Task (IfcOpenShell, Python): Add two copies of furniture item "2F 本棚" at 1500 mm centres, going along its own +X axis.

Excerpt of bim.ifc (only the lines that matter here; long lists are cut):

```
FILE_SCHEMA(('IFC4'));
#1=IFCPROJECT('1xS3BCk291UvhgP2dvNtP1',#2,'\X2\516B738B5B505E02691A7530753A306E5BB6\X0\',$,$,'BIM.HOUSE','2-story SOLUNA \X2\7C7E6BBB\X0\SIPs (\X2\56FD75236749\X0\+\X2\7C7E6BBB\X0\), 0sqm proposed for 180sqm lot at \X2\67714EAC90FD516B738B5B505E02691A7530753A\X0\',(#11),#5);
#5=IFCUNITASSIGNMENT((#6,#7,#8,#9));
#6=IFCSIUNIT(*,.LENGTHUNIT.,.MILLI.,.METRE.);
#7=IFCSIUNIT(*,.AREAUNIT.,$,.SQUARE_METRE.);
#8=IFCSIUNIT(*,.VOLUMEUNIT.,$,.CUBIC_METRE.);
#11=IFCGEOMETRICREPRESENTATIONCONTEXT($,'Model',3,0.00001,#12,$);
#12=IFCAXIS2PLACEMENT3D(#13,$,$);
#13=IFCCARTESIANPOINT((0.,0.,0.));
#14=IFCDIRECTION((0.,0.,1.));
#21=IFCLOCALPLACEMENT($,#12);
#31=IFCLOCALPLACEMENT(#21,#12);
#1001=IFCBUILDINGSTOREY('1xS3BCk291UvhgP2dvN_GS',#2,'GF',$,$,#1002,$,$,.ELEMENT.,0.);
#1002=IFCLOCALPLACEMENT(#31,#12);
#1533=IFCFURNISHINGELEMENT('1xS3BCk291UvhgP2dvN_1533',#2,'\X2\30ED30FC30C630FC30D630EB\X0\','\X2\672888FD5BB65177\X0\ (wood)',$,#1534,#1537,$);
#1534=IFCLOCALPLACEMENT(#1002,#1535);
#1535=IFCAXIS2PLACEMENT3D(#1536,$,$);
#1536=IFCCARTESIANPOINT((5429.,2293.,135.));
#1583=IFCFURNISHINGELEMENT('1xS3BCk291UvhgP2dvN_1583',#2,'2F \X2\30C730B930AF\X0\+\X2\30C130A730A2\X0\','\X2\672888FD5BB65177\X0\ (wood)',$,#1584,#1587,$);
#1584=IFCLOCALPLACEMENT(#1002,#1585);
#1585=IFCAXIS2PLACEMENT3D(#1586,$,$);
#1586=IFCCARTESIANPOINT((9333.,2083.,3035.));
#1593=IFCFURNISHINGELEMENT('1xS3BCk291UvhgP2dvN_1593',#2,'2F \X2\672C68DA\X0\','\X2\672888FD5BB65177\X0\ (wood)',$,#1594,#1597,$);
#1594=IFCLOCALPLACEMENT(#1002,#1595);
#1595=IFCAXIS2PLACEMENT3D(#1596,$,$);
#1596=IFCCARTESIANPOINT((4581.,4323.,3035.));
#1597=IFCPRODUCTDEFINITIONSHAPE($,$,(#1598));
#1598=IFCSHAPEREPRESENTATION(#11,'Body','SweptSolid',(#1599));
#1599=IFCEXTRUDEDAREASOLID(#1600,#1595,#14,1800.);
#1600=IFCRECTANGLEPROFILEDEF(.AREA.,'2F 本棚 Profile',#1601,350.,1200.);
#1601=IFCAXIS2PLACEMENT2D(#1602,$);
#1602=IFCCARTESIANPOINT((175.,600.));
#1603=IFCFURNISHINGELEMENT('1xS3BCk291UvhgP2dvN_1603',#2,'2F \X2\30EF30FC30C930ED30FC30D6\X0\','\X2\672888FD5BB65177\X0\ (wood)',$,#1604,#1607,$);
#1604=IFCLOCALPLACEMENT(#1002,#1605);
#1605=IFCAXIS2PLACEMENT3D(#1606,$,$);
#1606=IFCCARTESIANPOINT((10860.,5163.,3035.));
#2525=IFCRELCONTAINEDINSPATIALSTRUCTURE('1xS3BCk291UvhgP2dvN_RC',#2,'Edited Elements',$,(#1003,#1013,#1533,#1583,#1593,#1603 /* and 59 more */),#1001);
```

```python
import ifcopenshell
import ifcopenshell.api.geometry
import ifcopenshell.api.root
import ifcopenshell.util.element
import ifcopenshell.util.placement

model = ifcopenshell.open("bim.ifc")


def reuse_history(source, copy):
    """copy_class also copies each property set's owner history, people and application; keep the originals."""
    for rel in copy.IsDefinedBy:
        if rel.is_a("IfcRelDefinesByProperties") and (history := rel.RelatingPropertyDefinition.OwnerHistory):
            rel.RelatingPropertyDefinition.OwnerHistory = source.OwnerHistory
            ifcopenshell.util.element.remove_deep2(model, history)


source = model.by_id(1593)
base = ifcopenshell.util.placement.get_local_placement(source.ObjectPlacement)
step = base[:3, 0] * 1500.0

for i in range(1, 3):
    copy = ifcopenshell.api.root.copy_class(model, product=source)
    copy.Representation = ifcopenshell.util.element.copy_deep(
        model, source.Representation, exclude=["IfcGeometricRepresentationContext", "IfcRepresentationMap"]
    )
    reuse_history(source, copy)
    matrix = base.copy()
    matrix[:3, 3] += i * step
    print("added at", matrix[:3, 3].round(3) + 0.0)
    ifcopenshell.api.geometry.edit_object_placement(model, product=copy, matrix=matrix, is_si=False)

model.write("bim_v2.ifc")
```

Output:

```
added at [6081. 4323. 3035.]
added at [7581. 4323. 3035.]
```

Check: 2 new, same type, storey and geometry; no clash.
